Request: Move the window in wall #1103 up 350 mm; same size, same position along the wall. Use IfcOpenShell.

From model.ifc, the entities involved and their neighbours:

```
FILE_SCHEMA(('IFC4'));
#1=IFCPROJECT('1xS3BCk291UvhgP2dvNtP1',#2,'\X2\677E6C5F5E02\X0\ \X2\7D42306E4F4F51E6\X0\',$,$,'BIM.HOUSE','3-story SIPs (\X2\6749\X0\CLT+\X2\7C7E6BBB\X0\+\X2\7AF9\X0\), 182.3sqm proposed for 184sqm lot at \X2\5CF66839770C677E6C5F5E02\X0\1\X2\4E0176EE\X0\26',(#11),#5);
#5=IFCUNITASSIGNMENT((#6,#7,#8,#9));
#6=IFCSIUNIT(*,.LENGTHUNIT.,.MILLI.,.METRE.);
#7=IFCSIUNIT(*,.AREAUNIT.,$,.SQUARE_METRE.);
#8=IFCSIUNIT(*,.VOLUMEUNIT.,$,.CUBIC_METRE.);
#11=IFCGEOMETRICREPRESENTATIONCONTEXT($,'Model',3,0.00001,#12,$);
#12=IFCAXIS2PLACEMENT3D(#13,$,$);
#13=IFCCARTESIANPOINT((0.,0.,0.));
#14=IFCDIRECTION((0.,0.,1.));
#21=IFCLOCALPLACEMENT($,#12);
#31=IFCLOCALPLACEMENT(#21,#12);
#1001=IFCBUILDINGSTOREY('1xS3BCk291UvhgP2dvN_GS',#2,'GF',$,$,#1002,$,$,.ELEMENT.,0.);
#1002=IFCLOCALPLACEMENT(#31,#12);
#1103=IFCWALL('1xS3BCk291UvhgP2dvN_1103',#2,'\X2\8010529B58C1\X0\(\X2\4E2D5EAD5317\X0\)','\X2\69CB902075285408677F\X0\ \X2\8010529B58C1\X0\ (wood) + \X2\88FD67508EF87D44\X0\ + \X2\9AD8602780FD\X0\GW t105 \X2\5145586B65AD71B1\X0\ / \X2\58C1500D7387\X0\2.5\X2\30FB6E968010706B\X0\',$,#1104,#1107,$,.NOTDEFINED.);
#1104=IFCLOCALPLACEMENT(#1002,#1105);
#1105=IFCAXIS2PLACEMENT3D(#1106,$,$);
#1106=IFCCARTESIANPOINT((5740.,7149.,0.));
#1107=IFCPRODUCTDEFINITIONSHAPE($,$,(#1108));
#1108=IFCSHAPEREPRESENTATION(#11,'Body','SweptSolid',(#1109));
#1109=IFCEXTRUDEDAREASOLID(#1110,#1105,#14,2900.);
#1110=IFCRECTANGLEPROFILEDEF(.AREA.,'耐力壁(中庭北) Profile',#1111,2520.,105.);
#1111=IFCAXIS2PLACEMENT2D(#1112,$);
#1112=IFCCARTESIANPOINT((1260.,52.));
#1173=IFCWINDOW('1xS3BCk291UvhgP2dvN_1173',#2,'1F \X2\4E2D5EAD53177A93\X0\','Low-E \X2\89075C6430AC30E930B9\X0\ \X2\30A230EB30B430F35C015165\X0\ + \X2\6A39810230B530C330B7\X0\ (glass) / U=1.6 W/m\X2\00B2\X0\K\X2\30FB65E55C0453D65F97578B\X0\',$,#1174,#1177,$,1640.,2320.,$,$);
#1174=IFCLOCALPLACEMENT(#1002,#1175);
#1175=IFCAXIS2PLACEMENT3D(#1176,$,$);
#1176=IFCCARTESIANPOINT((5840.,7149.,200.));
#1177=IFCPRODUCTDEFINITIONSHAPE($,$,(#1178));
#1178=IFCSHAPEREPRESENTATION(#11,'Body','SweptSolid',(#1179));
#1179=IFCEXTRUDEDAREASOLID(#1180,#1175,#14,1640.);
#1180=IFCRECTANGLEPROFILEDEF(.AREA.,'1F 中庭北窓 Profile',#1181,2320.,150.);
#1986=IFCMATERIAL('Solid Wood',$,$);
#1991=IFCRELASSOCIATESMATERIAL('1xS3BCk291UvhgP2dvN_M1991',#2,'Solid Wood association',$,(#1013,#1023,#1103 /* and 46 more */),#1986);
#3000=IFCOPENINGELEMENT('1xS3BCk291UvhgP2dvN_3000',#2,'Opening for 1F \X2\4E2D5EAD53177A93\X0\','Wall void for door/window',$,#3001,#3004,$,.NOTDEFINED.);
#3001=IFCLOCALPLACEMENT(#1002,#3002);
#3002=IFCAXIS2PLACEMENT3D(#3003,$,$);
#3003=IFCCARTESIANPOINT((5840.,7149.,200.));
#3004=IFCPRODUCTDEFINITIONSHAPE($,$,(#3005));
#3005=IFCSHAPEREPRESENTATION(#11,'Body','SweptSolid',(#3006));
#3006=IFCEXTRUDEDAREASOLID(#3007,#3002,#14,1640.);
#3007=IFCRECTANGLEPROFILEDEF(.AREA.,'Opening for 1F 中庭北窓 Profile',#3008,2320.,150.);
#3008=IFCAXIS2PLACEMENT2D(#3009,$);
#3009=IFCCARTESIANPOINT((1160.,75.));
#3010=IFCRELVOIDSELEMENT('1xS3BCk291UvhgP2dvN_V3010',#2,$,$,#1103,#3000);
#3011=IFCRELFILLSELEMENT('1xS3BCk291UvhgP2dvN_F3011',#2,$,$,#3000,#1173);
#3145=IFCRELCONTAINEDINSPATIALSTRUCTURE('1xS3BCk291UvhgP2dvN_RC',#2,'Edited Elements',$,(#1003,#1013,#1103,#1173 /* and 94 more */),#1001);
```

```python
import numpy as np
import ifcopenshell
import ifcopenshell.api.geometry
import ifcopenshell.util.placement
import ifcopenshell.util.unit

model = ifcopenshell.open("model.ifc")
unit_scale = ifcopenshell.util.unit.calculate_unit_scale(model)

window = model.by_guid("1xS3BCk291UvhgP2dvN_1173")
opening = window.FillsVoids[0].RelatingOpeningElement
dz = 0.35 / unit_scale

shift = np.array([0.0, 0.0, dz])
# The window is not placed relative to its opening, so move both.
for product in (opening, window):
    matrix = ifcopenshell.util.placement.get_local_placement(product.ObjectPlacement)
    matrix[:3, 3] += shift
    ifcopenshell.api.geometry.edit_object_placement(model, product=product, matrix=matrix, is_si=False)

print(f"moved by {dz * unit_scale:+.3f} m")

model.write("model_rev.ifc")
```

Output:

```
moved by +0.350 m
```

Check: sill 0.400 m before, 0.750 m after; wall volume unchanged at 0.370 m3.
